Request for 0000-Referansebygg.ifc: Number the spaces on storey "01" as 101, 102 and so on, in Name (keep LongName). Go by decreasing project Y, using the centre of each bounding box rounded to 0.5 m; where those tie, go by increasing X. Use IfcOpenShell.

First a look at what the model holds.

```python
import ifcopenshell
import ifcopenshell.util.element
import ifcopenshell.util.placement

model = ifcopenshell.open("0000-Referansebygg.ifc")
print(model.schema)
storey = next(s for s in model.by_type("IfcBuildingStorey") if s.Name == "01")
spaces = [e for e in ifcopenshell.util.element.get_decomposition(storey) if e.is_a("IfcSpace")]
for e in sorted(spaces, key=lambda e: e.id()):
    origin = ifcopenshell.util.placement.get_local_placement(e.ObjectPlacement)[:3, 3]
    print(e.id(), e.Name, e.LongName, origin.round(2) + 0.0, sep=" | ")
```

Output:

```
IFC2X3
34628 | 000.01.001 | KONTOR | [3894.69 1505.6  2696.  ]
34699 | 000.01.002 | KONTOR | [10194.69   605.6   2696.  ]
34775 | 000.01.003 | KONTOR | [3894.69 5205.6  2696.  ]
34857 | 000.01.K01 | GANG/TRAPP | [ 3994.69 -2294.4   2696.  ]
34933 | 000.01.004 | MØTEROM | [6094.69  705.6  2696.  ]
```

```python
import ifcopenshell
import ifcopenshell.geom
import ifcopenshell.util.element
import ifcopenshell.util.shape

model = ifcopenshell.open("0000-Referansebygg.ifc")
settings = ifcopenshell.geom.settings()
settings.set("use-world-coords", True)


def centre(element):
    shape = ifcopenshell.geom.create_shape(settings, element)
    return ifcopenshell.util.shape.get_bbox_centroid(shape.geometry)


storey = next(s for s in model.by_type("IfcBuildingStorey") if s.Name == "01")
spaces = [e for e in ifcopenshell.util.element.get_decomposition(storey) if e.is_a("IfcSpace")]

# Insertion points can sit at a corner or the storey origin, so sort by the geometry (in metres).
centres = {e: centre(e) for e in spaces}
spaces.sort(key=lambda e: (-round(centres[e][1] / 0.5), centres[e][0]))

for i, e in enumerate(spaces, start=1):
    number = f"1{i:02d}"
    e.Name = number
    print(e.id(), number)

model.write("0000-Referansebygg_updated.ifc")
```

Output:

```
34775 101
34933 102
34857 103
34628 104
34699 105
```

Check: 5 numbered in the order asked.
